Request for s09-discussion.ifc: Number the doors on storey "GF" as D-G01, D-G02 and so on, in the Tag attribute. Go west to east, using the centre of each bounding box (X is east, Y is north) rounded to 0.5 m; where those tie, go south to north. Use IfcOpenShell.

First a look at what the model holds.

```python
import ifcopenshell
import ifcopenshell.util.element
import ifcopenshell.util.placement

model = ifcopenshell.open("s09-discussion.ifc")
print(model.schema)
storey = next(s for s in model.by_type("IfcBuildingStorey") if s.Name == "GF")
doors = [e for e in ifcopenshell.util.element.get_decomposition(storey) if e.is_a("IfcDoor")]
for e in sorted(doors, key=lambda e: e.id()):
    origin = ifcopenshell.util.placement.get_local_placement(e.ObjectPlacement)[:3, 3]
    print(e.id(), e.Tag, e.Name, origin.round(2) + 0.0, sep=" | ")
```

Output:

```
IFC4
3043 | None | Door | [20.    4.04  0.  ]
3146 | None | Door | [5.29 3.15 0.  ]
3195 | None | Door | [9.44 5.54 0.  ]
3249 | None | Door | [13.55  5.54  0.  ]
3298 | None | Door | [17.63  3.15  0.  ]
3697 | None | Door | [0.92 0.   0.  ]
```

```python
import ifcopenshell
import ifcopenshell.geom
import ifcopenshell.util.element
import ifcopenshell.util.shape

model = ifcopenshell.open("s09-discussion.ifc")
settings = ifcopenshell.geom.settings()
settings.set("use-world-coords", True)


def centre(element):
    shape = ifcopenshell.geom.create_shape(settings, element)
    return ifcopenshell.util.shape.get_bbox_centroid(shape.geometry)


storey = next(s for s in model.by_type("IfcBuildingStorey") if s.Name == "GF")
doors = [e for e in ifcopenshell.util.element.get_decomposition(storey) if e.is_a("IfcDoor")]

# Insertion points can sit at a corner or the storey origin, so sort by the geometry (in metres).
centres = {e: centre(e) for e in doors}
doors.sort(key=lambda e: (round(centres[e][0] / 0.5), centres[e][1]))

for i, e in enumerate(doors, start=1):
    number = f"D-G{i:02d}"
    e.Tag = number
    print(e.id(), number)

model.write("s09-discussion_edited.ifc")
```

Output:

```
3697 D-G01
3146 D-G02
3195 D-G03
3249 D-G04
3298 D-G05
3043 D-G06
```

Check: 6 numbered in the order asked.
